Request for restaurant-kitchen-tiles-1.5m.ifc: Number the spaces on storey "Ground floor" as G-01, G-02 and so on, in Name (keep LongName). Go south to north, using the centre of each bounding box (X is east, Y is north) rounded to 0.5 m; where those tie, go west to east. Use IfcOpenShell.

First a look at what the model holds.

```python
import ifcopenshell
import ifcopenshell.util.element
import ifcopenshell.util.placement

model = ifcopenshell.open("restaurant-kitchen-tiles-1.5m.ifc")
print(model.schema)
storey = next(s for s in model.by_type("IfcBuildingStorey") if s.Name == "Ground floor")
spaces = [e for e in ifcopenshell.util.element.get_decomposition(storey) if e.is_a("IfcSpace")]
for e in sorted(spaces, key=lambda e: e.id()):
    origin = ifcopenshell.util.placement.get_local_placement(e.ObjectPlacement)[:3, 3]
    print(e.id(), e.Name, e.LongName, origin.round(2) + 0.0, sep=" | ")
```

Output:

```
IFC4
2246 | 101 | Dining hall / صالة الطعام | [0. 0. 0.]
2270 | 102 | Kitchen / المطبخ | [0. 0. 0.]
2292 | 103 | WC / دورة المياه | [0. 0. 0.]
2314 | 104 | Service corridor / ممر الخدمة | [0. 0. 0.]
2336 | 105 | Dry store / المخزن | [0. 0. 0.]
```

```python
import ifcopenshell
import ifcopenshell.geom
import ifcopenshell.util.element
import ifcopenshell.util.shape

model = ifcopenshell.open("restaurant-kitchen-tiles-1.5m.ifc")
settings = ifcopenshell.geom.settings()
settings.set("use-world-coords", True)


def centre(element):
    shape = ifcopenshell.geom.create_shape(settings, element)
    return ifcopenshell.util.shape.get_bbox_centroid(shape.geometry)


storey = next(s for s in model.by_type("IfcBuildingStorey") if s.Name == "Ground floor")
spaces = [e for e in ifcopenshell.util.element.get_decomposition(storey) if e.is_a("IfcSpace")]

# Insertion points can sit at a corner or the storey origin, so sort by the geometry (in metres).
centres = {e: centre(e) for e in spaces}
spaces.sort(key=lambda e: (round(centres[e][1] / 0.5), centres[e][0]))

for i, e in enumerate(spaces, start=1):
    number = f"G-{i:02d}"
    e.Name = number
    print(e.id(), number)

model.write("restaurant-kitchen-tiles-1.5m_updated.ifc")
```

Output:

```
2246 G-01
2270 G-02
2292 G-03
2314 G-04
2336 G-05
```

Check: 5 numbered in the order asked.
